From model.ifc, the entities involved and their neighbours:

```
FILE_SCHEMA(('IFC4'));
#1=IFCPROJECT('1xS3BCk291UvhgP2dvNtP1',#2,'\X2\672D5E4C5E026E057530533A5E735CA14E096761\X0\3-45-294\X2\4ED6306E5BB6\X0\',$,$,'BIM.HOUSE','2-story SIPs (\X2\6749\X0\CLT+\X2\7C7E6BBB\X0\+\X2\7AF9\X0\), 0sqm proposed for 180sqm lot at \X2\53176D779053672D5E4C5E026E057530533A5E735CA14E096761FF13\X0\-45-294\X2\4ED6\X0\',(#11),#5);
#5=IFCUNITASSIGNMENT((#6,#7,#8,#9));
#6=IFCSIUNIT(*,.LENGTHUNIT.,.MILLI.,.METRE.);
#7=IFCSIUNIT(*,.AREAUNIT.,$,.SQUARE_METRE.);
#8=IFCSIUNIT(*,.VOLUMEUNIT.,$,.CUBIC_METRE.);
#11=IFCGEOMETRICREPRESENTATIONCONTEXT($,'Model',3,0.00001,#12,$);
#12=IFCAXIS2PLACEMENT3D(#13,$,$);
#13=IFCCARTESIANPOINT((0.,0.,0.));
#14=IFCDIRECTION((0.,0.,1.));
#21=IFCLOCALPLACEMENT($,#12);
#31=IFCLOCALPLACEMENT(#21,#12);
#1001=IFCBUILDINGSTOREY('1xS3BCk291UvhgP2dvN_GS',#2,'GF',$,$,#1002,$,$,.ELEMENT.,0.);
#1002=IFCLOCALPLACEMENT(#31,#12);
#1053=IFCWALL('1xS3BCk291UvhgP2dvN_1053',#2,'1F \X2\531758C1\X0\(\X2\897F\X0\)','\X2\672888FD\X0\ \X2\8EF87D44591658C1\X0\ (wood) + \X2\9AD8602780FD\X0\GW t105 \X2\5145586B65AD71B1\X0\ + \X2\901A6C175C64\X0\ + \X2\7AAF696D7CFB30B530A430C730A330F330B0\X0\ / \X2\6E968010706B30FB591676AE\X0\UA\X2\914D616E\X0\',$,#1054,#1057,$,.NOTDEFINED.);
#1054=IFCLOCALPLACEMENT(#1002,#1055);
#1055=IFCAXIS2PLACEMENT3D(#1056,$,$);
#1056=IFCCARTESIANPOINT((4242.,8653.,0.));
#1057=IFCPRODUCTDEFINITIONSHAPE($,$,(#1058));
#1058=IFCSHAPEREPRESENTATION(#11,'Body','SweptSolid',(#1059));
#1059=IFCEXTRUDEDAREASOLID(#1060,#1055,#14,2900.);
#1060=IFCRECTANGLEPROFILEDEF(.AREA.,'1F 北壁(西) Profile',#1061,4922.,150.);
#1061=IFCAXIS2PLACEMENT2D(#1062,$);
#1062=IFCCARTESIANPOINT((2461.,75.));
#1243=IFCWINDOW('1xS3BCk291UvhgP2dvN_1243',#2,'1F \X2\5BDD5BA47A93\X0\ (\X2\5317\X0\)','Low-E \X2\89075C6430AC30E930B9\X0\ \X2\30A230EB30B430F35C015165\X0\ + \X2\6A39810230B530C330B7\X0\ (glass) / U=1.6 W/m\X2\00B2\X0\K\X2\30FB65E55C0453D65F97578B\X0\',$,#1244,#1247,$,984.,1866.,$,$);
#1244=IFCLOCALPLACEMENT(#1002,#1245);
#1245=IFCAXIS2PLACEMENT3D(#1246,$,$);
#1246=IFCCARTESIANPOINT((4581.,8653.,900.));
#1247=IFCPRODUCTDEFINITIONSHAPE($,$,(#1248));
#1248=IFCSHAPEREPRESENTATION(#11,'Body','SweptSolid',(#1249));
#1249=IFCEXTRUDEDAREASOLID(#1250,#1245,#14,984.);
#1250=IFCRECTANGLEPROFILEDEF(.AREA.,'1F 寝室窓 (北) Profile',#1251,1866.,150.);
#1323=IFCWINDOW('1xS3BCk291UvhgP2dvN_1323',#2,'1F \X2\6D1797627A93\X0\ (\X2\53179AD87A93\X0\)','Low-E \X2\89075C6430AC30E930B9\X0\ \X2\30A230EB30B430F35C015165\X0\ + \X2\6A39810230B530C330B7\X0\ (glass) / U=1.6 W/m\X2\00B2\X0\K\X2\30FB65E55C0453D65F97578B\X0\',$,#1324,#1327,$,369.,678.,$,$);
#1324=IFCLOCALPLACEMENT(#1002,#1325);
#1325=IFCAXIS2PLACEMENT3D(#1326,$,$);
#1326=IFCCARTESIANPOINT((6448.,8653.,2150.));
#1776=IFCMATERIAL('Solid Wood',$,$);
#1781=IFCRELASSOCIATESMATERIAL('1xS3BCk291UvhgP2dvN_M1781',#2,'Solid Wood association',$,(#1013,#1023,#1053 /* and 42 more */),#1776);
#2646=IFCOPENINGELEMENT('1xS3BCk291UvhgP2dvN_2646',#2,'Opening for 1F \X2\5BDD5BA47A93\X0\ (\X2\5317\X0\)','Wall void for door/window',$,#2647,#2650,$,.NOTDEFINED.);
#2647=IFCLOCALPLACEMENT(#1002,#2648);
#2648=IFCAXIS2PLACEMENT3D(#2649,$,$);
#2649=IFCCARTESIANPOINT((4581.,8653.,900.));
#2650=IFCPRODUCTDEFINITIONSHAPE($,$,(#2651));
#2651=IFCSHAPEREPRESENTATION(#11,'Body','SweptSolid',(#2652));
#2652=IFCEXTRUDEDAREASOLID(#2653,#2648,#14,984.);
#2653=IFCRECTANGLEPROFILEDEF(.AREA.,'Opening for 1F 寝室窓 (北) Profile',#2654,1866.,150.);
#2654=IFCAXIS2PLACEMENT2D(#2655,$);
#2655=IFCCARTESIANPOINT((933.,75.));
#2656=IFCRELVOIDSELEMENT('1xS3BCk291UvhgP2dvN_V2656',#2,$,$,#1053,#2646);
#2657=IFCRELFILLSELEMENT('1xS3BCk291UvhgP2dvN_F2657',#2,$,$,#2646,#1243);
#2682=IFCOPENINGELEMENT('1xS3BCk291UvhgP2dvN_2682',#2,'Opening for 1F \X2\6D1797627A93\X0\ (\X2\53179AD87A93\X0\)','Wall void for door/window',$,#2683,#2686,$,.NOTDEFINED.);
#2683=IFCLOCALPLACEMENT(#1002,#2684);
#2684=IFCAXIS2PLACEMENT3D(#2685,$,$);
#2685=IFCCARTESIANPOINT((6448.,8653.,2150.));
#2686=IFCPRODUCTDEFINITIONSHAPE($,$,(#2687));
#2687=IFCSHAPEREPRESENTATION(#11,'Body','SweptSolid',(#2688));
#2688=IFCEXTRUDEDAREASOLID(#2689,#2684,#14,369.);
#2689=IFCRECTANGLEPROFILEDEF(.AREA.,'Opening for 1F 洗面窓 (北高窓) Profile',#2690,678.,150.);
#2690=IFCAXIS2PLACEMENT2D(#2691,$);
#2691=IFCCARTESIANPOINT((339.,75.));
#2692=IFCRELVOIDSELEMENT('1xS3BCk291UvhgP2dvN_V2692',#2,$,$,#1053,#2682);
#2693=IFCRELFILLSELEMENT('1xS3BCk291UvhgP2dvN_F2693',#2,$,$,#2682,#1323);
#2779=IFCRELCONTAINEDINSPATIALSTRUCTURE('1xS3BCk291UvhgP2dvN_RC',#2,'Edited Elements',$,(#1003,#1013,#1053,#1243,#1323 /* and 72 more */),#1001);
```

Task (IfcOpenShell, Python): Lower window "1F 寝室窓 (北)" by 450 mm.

```python
import numpy as np
import ifcopenshell
import ifcopenshell.api.geometry
import ifcopenshell.util.placement
import ifcopenshell.util.unit

model = ifcopenshell.open("model.ifc")
unit_scale = ifcopenshell.util.unit.calculate_unit_scale(model)

window = model.by_guid("1xS3BCk291UvhgP2dvN_1243")
opening = window.FillsVoids[0].RelatingOpeningElement
dz = -0.45 / unit_scale

shift = np.array([0.0, 0.0, dz])
# The window is not placed relative to its opening, so move both.
for product in (opening, window):
    matrix = ifcopenshell.util.placement.get_local_placement(product.ObjectPlacement)
    matrix[:3, 3] += shift
    ifcopenshell.api.geometry.edit_object_placement(model, product=product, matrix=matrix, is_si=False)

print(f"moved by {dz * unit_scale:+.3f} m")

model.write("model_rev.ifc")
```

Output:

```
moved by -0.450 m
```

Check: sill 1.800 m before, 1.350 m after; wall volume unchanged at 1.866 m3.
